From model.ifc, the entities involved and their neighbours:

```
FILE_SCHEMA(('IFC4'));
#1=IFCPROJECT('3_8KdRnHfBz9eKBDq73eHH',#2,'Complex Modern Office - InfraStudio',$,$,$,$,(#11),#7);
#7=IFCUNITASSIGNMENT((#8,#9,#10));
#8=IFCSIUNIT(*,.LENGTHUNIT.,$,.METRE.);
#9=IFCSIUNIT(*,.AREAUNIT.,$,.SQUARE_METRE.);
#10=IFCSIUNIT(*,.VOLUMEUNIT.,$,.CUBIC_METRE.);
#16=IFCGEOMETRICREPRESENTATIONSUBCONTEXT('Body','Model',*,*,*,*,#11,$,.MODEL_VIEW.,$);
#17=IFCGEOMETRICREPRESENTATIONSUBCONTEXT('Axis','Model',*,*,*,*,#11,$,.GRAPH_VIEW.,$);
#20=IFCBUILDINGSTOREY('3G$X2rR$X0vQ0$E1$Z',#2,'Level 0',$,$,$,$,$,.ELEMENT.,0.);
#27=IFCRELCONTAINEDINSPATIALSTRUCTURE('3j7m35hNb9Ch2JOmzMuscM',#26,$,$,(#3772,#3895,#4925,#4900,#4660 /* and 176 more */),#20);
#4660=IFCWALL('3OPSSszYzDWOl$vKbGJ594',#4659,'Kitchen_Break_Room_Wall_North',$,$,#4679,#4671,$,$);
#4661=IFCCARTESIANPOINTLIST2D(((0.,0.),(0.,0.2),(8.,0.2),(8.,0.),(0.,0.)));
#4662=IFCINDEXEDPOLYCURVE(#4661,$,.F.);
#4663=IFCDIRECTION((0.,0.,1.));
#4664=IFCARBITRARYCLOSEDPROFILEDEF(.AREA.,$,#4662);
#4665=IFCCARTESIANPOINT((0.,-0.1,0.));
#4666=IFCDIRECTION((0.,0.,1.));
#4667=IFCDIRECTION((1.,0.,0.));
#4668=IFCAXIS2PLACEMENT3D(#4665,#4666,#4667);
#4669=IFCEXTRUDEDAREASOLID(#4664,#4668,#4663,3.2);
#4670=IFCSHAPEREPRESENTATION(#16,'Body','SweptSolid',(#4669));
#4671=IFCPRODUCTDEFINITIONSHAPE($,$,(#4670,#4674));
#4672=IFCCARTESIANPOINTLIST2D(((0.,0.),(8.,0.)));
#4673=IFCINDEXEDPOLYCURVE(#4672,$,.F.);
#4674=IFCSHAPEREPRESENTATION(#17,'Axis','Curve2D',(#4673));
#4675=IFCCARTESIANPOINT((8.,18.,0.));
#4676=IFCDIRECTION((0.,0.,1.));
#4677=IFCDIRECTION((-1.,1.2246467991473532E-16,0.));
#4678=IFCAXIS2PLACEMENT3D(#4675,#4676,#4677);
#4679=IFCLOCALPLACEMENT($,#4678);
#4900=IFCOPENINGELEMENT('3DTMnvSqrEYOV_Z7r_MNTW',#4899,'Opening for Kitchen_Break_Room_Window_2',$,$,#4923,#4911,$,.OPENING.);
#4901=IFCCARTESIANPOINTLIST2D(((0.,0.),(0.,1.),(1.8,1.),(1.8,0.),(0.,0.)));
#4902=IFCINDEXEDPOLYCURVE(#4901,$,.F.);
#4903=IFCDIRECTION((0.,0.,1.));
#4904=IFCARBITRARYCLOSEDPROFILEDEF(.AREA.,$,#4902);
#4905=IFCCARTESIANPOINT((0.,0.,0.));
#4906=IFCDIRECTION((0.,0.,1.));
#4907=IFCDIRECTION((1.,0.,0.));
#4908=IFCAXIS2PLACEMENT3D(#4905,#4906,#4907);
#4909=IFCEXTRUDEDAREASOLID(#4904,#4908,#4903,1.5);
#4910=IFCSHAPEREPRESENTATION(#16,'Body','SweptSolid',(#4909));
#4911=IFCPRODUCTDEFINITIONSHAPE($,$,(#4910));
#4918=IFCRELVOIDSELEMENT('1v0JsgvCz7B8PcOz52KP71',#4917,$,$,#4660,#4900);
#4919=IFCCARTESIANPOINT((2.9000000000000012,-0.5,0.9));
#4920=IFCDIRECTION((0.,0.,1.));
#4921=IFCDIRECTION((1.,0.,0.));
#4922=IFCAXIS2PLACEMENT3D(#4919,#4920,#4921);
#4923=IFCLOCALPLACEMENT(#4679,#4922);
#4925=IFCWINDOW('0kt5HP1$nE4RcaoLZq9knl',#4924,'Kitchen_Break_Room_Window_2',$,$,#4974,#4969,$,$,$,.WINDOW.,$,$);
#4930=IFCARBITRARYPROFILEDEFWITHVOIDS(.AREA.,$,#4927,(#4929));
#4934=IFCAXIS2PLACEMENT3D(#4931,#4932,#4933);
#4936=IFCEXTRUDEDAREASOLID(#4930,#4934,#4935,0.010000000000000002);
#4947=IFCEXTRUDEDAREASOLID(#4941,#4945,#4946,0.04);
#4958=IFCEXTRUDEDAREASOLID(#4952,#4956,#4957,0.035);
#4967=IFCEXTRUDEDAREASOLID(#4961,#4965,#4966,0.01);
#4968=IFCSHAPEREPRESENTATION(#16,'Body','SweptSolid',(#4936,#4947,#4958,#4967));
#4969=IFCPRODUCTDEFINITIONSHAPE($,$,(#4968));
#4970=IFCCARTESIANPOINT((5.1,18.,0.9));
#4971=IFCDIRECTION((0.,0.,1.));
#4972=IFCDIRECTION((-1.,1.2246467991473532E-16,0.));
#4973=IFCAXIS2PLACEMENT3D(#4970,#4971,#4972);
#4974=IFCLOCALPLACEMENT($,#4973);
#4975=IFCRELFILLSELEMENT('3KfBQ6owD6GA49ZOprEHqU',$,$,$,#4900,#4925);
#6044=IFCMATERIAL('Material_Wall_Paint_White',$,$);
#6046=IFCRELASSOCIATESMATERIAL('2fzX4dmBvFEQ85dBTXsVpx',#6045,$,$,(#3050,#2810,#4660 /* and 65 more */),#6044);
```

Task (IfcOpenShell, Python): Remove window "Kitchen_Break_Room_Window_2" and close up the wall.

```python
import ifcopenshell
import ifcopenshell.api.feature
import ifcopenshell.api.root
import ifcopenshell.geom
import ifcopenshell.util.shape

model = ifcopenshell.open("model.ifc")
settings = ifcopenshell.geom.settings()


def volume(element):
    """Net volume in cubic metres, openings subtracted."""
    shape = ifcopenshell.geom.create_shape(settings, element)
    return ifcopenshell.util.shape.get_volume(shape.geometry)


window = model.by_guid("0kt5HP1$nE4RcaoLZq9knl")
opening = window.FillsVoids[0].RelatingOpeningElement
wall = opening.VoidsElements[0].RelatingBuildingElement
before = volume(wall)

ifcopenshell.api.root.remove_product(model, product=window)
ifcopenshell.api.feature.remove_feature(model, feature=opening)

after = volume(wall)

print(f"wall volume {before:.3f} -> {after:.3f} m3")

model.write("model_v2.ifc")
```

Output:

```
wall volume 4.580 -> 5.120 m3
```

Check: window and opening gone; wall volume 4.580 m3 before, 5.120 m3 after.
